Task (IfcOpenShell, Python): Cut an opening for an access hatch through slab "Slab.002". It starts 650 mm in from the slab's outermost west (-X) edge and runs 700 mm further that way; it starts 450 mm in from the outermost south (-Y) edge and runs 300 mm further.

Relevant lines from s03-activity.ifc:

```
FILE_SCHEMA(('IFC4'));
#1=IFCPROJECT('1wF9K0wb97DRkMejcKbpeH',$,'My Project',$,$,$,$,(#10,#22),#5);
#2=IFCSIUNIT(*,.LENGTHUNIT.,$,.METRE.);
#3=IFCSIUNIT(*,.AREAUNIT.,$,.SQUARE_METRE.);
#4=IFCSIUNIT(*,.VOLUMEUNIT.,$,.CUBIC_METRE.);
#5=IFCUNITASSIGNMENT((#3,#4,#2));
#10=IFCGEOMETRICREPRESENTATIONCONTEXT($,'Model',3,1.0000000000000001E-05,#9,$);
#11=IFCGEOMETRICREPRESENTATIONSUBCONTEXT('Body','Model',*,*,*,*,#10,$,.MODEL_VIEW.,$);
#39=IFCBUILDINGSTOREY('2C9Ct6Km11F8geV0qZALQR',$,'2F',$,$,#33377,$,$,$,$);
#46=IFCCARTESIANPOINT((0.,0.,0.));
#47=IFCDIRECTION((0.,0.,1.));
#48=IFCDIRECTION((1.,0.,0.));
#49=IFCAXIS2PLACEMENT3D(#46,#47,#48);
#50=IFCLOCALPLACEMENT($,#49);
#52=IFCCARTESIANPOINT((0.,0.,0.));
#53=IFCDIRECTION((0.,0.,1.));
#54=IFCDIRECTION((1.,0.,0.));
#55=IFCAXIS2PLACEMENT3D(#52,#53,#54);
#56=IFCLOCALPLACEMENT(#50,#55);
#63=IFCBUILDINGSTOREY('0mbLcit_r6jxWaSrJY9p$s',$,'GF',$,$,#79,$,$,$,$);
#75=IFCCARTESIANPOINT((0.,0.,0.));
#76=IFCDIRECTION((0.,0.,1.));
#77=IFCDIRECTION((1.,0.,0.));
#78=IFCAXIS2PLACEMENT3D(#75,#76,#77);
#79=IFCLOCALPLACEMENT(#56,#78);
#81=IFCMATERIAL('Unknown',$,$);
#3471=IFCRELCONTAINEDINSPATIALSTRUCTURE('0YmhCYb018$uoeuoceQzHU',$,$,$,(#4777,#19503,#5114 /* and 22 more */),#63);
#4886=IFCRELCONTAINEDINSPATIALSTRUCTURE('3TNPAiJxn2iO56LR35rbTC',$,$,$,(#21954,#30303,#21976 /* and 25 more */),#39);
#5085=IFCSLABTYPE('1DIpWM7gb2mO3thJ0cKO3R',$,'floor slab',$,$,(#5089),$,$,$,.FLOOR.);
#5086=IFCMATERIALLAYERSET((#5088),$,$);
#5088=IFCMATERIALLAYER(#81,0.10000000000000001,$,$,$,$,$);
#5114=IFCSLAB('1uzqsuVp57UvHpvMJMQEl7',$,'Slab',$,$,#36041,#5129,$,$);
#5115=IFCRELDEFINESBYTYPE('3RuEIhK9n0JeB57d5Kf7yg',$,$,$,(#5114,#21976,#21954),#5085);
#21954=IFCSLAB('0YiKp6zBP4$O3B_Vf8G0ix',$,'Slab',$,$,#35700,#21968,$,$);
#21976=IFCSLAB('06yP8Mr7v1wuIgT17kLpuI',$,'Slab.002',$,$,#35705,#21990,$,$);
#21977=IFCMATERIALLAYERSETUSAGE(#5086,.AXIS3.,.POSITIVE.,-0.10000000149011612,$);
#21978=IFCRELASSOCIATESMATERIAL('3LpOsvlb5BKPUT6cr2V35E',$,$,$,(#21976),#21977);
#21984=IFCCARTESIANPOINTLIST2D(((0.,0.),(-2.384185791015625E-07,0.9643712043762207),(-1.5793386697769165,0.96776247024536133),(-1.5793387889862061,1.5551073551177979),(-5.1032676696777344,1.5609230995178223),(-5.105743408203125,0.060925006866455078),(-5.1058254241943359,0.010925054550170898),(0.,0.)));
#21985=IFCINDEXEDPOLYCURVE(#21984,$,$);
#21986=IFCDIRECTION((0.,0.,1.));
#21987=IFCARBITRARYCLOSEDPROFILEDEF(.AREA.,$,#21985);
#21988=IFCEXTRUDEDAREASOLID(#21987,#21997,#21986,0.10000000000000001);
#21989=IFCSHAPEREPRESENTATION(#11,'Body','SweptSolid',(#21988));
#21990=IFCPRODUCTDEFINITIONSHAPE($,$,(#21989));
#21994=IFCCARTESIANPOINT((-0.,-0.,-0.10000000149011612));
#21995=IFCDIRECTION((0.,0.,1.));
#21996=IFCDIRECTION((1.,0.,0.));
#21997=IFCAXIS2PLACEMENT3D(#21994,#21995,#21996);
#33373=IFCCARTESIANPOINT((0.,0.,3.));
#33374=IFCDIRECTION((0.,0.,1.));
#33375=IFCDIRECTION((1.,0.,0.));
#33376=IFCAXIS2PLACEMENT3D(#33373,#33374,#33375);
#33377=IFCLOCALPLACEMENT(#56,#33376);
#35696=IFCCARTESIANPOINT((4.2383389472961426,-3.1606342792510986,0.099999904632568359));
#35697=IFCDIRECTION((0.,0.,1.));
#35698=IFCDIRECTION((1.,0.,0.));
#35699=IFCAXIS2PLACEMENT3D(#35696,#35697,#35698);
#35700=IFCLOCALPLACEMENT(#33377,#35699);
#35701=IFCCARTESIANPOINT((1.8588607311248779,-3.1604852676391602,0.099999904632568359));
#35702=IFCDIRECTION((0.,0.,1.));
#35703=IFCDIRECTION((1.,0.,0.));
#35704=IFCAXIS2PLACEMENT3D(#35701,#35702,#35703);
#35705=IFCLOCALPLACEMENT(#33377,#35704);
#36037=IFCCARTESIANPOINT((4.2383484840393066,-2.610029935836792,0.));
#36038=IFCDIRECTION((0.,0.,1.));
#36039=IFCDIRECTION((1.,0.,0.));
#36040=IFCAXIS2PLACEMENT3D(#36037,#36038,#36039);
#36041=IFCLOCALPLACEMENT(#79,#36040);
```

```python
import numpy as np
import ifcopenshell
import ifcopenshell.api.feature
import ifcopenshell.api.geometry
import ifcopenshell.api.root
import ifcopenshell.geom
import ifcopenshell.util.placement
import ifcopenshell.util.representation
import ifcopenshell.util.shape
import ifcopenshell.util.unit

model = ifcopenshell.open("s03-activity.ifc")
unit_scale = ifcopenshell.util.unit.calculate_unit_scale(model)
settings = ifcopenshell.geom.settings()


def volume(element):
    """Net volume in cubic metres, openings subtracted."""
    shape = ifcopenshell.geom.create_shape(settings, element)
    return ifcopenshell.util.shape.get_volume(shape.geometry)


slab = model.by_id(21976)
before = volume(slab)

# Extent in the slab's own axes, in metres. The edges named are its -X and -Y sides.
slab_shape = ifcopenshell.geom.create_shape(settings, slab)
vertices = ifcopenshell.util.shape.get_vertices(slab_shape.geometry)
x_min, y_min, bottom = vertices.min(axis=0)
top = vertices[:, 2].max()

opening = ifcopenshell.api.root.create_entity(model, ifc_class="IfcOpeningElement", name="Access hatch opening", predefined_type="OPENING")
context = ifcopenshell.util.representation.get_context(model, "Model", "Body", "MODEL_VIEW")
width, depth = 0.7, 0.3
outline = [(0.0, 0.0), (width, 0.0), (width, depth), (0.0, depth), (0.0, 0.0)]
# Overshoot both faces by 50 mm so the cut is clean.
shape = ifcopenshell.api.geometry.add_slab_representation(
    model, context=context, depth=top - bottom + 0.1, polyline=outline
)
ifcopenshell.api.geometry.assign_representation(model, product=opening, representation=shape)

matrix = ifcopenshell.util.placement.get_local_placement(slab.ObjectPlacement)
matrix[:, 3] = matrix @ np.append(np.array([x_min + 0.65, y_min + 0.45, bottom - 0.05]) / unit_scale, 1.0)
ifcopenshell.api.geometry.edit_object_placement(model, product=opening, matrix=matrix, is_si=False)
ifcopenshell.api.feature.add_feature(model, feature=opening, element=slab)

after = volume(slab)

print(f"slab volume {before:.3f} -> {after:.3f} m3")

model.write("s03-activity_edited.ifc")
```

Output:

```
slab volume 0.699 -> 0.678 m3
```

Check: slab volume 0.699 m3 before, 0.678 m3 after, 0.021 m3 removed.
